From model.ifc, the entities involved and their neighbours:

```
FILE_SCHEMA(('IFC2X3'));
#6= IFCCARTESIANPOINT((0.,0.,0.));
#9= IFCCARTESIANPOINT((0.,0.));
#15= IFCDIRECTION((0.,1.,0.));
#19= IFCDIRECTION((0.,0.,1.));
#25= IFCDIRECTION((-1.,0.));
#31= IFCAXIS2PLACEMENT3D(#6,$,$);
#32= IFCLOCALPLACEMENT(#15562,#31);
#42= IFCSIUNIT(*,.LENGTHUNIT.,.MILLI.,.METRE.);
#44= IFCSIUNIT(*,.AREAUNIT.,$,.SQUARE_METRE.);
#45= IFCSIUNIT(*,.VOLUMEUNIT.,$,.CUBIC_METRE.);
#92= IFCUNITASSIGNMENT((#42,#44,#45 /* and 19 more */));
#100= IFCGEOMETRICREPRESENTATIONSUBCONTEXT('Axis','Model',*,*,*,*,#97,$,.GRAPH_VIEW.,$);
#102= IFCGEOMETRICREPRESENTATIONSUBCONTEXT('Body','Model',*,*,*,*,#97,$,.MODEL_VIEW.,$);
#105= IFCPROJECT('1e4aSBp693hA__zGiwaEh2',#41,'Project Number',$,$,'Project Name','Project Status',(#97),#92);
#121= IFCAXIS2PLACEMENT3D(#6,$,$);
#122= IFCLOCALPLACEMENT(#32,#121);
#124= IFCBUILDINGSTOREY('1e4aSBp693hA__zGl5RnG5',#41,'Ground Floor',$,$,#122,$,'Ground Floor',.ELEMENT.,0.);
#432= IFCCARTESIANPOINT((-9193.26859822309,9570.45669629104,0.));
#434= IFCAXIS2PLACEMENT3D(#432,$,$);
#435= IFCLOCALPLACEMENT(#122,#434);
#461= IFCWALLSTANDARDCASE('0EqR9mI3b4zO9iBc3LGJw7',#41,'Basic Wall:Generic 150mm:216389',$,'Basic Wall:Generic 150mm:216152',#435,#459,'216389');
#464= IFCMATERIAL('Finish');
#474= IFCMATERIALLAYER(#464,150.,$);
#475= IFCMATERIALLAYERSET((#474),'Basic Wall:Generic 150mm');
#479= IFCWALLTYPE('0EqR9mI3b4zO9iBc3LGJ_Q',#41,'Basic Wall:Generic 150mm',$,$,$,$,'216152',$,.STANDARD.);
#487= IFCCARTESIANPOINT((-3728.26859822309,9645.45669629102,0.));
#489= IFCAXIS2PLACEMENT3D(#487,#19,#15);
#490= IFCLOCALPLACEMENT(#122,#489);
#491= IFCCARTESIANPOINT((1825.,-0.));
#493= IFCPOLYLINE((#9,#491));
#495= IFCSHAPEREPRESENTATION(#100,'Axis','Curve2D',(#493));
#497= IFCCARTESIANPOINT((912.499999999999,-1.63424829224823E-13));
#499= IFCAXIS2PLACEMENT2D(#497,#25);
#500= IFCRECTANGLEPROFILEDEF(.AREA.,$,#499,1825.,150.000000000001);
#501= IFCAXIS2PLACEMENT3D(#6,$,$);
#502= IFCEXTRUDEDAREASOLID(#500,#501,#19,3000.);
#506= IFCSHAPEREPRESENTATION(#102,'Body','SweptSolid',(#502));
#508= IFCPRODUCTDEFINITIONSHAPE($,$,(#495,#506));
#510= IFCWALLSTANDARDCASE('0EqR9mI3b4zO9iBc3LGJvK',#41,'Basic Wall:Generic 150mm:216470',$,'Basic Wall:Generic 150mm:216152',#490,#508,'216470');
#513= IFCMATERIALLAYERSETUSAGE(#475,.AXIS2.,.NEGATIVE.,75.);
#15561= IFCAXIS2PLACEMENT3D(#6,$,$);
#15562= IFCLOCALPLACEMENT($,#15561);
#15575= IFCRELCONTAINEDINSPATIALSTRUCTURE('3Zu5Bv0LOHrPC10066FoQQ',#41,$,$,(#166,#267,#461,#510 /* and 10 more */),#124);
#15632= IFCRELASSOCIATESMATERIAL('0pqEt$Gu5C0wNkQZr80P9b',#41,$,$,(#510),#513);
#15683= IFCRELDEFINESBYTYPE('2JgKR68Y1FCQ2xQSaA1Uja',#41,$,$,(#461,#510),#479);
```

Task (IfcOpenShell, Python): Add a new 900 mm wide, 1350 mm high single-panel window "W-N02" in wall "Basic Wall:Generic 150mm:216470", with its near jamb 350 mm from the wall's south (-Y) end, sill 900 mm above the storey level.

```python
import numpy as np
import ifcopenshell
import ifcopenshell.api.feature
import ifcopenshell.api.geometry
import ifcopenshell.api.root
import ifcopenshell.api.spatial
import ifcopenshell.api.type
import ifcopenshell.geom
import ifcopenshell.util.element
import ifcopenshell.util.placement
import ifcopenshell.util.representation
import ifcopenshell.util.shape
import ifcopenshell.util.unit

model = ifcopenshell.open("model.ifc")
unit_scale = ifcopenshell.util.unit.calculate_unit_scale(model)
settings = ifcopenshell.geom.settings()


def volume(element):
    """Net volume in cubic metres, openings subtracted."""
    shape = ifcopenshell.geom.create_shape(settings, element)
    return ifcopenshell.util.shape.get_volume(shape.geometry)


wall = model.by_id(510)
storey = ifcopenshell.util.element.get_container(wall, ifc_class="IfcBuildingStorey")
context = ifcopenshell.util.representation.get_context(model, "Model", "Body", "MODEL_VIEW")
before = volume(wall)

width, height, from_end, sill = 0.9, 1.35, 0.35, 0.9  # metres

# The wall runs along its own X axis, and the end named is its -X end.
wall_shape = ifcopenshell.geom.create_shape(settings, wall)
x, y, z = ifcopenshell.util.shape.get_vertices(wall_shape.geometry).T
start = x.min() + from_end
face, thickness = float(y.min()), float(y.max() - y.min())
wall_matrix = ifcopenshell.util.placement.get_local_placement(wall.ObjectPlacement)
level = ifcopenshell.util.placement.get_local_placement(storey.ObjectPlacement)[2, 3]


def in_wall(x, y):
    """Placement at x, y metres in the wall's axes, at sill height."""
    matrix = wall_matrix.copy()
    matrix[:, 3] = wall_matrix @ np.array([x / unit_scale, y / unit_scale, 0.0, 1.0])
    matrix[2, 3] = level + sill / unit_scale
    return matrix


# Opening: a box that overshoots both wall faces by 50 mm.
opening = ifcopenshell.api.root.create_entity(model, ifc_class="IfcOpeningElement")
box = ifcopenshell.api.geometry.add_wall_representation(
    model, context=context, length=width, height=height, thickness=thickness + 0.1
)
ifcopenshell.api.geometry.assign_representation(model, product=opening, representation=box)
ifcopenshell.api.geometry.edit_object_placement(model, product=opening, matrix=in_wall(start, face - 0.05), is_si=False)
ifcopenshell.api.feature.add_feature(model, feature=opening, element=wall)

window = ifcopenshell.api.root.create_entity(model, ifc_class="IfcWindow", name="W-N02")
window.OverallWidth, window.OverallHeight = width / unit_scale, height / unit_scale
body = ifcopenshell.api.geometry.add_window_representation(
    model,
    context=context,
    overall_width=window.OverallWidth,
    overall_height=window.OverallHeight,
    partition_type="SINGLE_PANEL",
)
ifcopenshell.api.geometry.assign_representation(model, product=window, representation=body)
ifcopenshell.api.spatial.assign_container(model, products=[window], relating_structure=storey)
fills = ifcopenshell.api.feature.add_filling(model, opening=opening, element=window)
fills.OwnerHistory = window.OwnerHistory  # required in IFC2X3

# IFC2X3 keeps the operation on the window style.
style = ifcopenshell.api.root.create_entity(model, ifc_class="IfcWindowStyle", name="W-N02")
style.OperationType, style.ConstructionType = "SINGLE_PANEL", "NOTDEFINED"
style.ParameterTakesPrecedence = style.Sizeable = False
ifcopenshell.api.type.assign_type(model, related_objects=[window], relating_type=style)

# Centre the window in the wall's thickness.
ifcopenshell.api.geometry.edit_object_placement(model, product=window, matrix=in_wall(start, face), is_si=False)
window_shape = ifcopenshell.geom.create_shape(settings, window)
depth = ifcopenshell.util.shape.get_vertices(window_shape.geometry)[:, 1]
offset = face + thickness / 2 - (depth.min() + depth.max()) / 2
ifcopenshell.api.geometry.edit_object_placement(model, product=window, matrix=in_wall(start, offset), is_si=False)

after = volume(wall)

print(f"wall volume {before:.3f} -> {after:.3f} m3")

model.write("model_v2.ifc")
```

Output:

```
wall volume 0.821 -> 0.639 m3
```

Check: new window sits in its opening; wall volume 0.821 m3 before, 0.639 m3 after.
